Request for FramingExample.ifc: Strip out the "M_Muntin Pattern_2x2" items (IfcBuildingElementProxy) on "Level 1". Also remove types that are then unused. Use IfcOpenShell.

First a look at what the model holds.

```python
import ifcopenshell
import ifcopenshell.util.element

model = ifcopenshell.open("FramingExample.ifc")
print(model.schema)
storey = next(s for s in model.by_type("IfcBuildingStorey") if s.Name == "Level 1")
proxies = [e for e in ifcopenshell.util.element.get_decomposition(storey) if e.is_a("IfcBuildingElementProxy")]
seen = {}
for e in proxies:
    element_type = ifcopenshell.util.element.get_type(e)
    name = element_type.Name if element_type not in (None, e) else None
    seen[name] = seen.get(name, 0) + 1
for name, count in sorted(seen.items(), key=str):
    print(count, "x", name)
```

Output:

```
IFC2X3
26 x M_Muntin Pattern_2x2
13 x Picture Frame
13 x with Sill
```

```python
import ifcopenshell
import ifcopenshell.api.root
import ifcopenshell.util.element

model = ifcopenshell.open("FramingExample.ifc")

storey = next(s for s in model.by_type("IfcBuildingStorey") if s.Name == "Level 1")
proxies = [e for e in ifcopenshell.util.element.get_decomposition(storey) if e.is_a("IfcBuildingElementProxy")]
targets = [e for e in proxies if (t := ifcopenshell.util.element.get_type(e)) not in (None, e) and t.Name == "M_Muntin Pattern_2x2"]
types = {ifcopenshell.util.element.get_type(e) for e in targets} - {None, *targets}

for e in targets:
    ifcopenshell.api.root.remove_product(model, product=e)
print(len(targets), "removed")

unused = [t for t in types if not ifcopenshell.util.element.get_types(t)]
for t in unused:
    ifcopenshell.api.root.remove_product(model, product=t)
print(len(unused), "unused types removed")

model.write("FramingExample_v2.ifc")
```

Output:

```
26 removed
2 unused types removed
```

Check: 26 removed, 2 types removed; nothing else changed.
